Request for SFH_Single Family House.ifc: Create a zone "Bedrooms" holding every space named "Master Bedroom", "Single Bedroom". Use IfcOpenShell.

First a look at what the model holds.

```python
import ifcopenshell

model = ifcopenshell.open("SFH_Single Family House.ifc")
print(model.schema)
seen = {}
for space in model.by_type("IfcSpace"):
    seen[space.LongName] = seen.get(space.LongName, 0) + 1
for name, count in sorted(seen.items(), key=str):
    print(count, "x", name)
print("zones:", [z.Name for z in model.by_type("IfcZone")][:20])
```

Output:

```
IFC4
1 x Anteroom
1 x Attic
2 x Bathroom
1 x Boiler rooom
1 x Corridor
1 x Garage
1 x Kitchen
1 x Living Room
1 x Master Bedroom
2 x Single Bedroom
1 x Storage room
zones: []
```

```python
import ifcopenshell
import ifcopenshell.api.group
import ifcopenshell.api.root

model = ifcopenshell.open("SFH_Single Family House.ifc")

names = {"Master Bedroom", "Single Bedroom"}
spaces = [s for s in model.by_type("IfcSpace") if s.LongName in names]

zone = ifcopenshell.api.root.create_entity(model, ifc_class="IfcZone", name="Bedrooms")
ifcopenshell.api.group.assign_group(model, products=spaces, group=zone)
print(len(spaces), "spaces in", zone.Name)

model.write("SFH_Single Family House_updated.ifc")
```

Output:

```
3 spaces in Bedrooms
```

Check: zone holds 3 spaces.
